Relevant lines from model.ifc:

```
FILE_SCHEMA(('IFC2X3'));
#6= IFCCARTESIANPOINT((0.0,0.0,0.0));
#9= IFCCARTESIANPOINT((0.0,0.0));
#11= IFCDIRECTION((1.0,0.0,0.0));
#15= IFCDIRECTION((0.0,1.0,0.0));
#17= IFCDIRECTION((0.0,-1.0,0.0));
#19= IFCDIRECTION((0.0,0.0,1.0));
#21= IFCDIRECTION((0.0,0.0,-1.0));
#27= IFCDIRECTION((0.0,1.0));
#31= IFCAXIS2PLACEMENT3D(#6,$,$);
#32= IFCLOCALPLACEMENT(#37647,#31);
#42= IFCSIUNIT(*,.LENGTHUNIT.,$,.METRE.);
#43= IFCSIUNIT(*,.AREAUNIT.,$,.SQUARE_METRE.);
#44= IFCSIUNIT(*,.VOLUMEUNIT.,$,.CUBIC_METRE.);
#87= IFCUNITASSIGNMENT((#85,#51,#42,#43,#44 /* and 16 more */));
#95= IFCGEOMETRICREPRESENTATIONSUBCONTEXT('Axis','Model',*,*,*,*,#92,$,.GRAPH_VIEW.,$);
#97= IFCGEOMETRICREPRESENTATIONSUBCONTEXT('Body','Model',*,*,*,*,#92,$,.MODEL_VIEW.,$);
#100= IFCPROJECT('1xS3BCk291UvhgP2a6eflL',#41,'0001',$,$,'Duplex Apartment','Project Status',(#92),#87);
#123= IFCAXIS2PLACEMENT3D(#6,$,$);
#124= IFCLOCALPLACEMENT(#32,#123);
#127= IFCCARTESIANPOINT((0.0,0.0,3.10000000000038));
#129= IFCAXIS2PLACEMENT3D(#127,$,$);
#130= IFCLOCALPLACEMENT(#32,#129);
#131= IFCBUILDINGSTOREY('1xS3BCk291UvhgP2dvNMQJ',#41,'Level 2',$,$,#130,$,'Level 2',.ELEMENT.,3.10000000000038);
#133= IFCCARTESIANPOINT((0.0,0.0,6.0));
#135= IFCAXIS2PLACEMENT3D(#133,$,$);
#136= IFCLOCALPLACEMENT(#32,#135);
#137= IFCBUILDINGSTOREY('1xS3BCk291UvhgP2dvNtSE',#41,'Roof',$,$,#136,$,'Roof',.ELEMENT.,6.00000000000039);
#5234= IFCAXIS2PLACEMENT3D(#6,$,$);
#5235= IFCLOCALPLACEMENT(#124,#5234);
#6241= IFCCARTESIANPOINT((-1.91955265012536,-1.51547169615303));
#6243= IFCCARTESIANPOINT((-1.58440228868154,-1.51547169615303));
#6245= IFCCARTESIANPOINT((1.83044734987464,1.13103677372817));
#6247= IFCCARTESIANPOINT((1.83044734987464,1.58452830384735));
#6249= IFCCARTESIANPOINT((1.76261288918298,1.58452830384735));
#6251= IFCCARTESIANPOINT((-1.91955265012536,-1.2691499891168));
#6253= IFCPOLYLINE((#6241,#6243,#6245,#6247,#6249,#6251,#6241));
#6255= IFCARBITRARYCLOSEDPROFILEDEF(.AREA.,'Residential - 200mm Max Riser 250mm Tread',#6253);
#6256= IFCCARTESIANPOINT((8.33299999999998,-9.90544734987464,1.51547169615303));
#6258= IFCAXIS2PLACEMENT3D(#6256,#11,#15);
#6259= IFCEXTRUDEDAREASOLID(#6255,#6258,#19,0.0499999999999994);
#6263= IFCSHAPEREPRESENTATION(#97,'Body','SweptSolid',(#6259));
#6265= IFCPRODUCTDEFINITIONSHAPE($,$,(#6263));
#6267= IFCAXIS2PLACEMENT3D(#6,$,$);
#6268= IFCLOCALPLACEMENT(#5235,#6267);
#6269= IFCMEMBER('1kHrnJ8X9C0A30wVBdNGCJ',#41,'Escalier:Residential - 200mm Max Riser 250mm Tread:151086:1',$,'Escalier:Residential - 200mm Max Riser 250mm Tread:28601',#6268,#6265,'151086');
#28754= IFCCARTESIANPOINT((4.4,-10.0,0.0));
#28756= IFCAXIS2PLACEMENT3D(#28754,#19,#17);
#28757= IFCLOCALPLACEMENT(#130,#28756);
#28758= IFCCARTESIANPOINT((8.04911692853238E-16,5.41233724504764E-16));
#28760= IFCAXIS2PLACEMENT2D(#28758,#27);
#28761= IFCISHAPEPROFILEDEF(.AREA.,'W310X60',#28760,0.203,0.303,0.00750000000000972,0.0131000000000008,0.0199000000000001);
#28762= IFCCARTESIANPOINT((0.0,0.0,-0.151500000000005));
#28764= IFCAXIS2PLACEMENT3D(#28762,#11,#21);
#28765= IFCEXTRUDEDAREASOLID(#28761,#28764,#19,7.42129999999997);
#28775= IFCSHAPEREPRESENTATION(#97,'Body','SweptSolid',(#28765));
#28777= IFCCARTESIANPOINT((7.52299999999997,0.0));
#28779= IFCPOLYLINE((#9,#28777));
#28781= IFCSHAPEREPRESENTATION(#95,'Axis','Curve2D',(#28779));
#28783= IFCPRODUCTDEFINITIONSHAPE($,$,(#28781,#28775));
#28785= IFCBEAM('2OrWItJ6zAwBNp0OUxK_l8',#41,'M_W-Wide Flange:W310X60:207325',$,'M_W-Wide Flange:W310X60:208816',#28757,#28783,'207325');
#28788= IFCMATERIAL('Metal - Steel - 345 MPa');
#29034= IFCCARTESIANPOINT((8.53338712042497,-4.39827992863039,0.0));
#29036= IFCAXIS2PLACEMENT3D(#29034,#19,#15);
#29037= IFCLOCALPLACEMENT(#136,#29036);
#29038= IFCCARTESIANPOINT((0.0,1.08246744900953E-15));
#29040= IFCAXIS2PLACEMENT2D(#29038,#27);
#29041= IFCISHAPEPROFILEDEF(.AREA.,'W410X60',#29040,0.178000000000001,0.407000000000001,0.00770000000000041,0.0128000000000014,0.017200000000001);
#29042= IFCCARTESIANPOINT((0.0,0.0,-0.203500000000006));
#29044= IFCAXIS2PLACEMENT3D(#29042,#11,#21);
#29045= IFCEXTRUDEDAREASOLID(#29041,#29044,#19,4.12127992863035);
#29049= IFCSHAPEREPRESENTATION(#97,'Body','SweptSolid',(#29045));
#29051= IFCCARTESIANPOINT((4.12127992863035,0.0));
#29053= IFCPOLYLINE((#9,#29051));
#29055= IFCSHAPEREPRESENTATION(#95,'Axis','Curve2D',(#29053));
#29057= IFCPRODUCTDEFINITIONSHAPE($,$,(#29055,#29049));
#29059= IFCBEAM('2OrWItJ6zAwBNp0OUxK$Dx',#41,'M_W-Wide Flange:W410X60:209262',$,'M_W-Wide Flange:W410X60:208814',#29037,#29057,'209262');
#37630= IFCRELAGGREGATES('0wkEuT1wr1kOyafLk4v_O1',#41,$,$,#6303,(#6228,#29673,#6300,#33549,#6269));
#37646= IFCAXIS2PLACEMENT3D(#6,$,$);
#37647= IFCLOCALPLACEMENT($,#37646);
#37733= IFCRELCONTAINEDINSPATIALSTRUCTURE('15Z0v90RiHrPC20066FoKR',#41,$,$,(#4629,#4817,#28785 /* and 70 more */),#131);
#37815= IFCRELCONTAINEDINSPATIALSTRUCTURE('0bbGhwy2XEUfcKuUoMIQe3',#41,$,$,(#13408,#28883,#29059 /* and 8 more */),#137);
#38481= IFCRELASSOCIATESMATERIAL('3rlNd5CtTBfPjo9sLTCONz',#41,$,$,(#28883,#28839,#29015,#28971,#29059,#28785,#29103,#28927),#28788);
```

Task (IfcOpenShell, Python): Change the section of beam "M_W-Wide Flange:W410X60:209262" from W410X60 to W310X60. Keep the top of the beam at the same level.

```python
import ifcopenshell
import ifcopenshell.util.element
import ifcopenshell.util.representation

model = ifcopenshell.open("model.ifc")

member = model.by_guid("2OrWItJ6zAwBNp0OUxK$Dx")
source = next(p for p in model.by_type("IfcIShapeProfileDef") if p.ProfileName == "W310X60")

body = ifcopenshell.util.representation.get_representation(member, "Model", "Body")
solid = body.Items[0]
old_profile = solid.SweptArea

# Copy the section's sizes but keep this member's own profile position.
profile = ifcopenshell.util.element.copy(model, source)
# Profiles are centred, so shift by half the change in depth to hold the top.
shift = (old_profile.OverallDepth - profile.OverallDepth) / 2
x, y = old_profile.Position.Location.Coordinates
up = (-1.0, 0.0)  # upwards, in the solid's own plane
location = model.createIfcCartesianPoint((x + up[0] * shift, y + up[1] * shift))
profile.Position = model.createIfcAxis2Placement2D(location, old_profile.Position.RefDirection)
solid.SweptArea = profile
if not model.get_total_inverses(old_profile):
    ifcopenshell.util.element.remove_deep2(model, old_profile)
member.Name = member.Name.replace("W410X60", "W310X60")
member.ObjectType = member.ObjectType.replace("W410X60", "W310X60")

print(solid.SweptArea)

model.write("model-out.ifc")
```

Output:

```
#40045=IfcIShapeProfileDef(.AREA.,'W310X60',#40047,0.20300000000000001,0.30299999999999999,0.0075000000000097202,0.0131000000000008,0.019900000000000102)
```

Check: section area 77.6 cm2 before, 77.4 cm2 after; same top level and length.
